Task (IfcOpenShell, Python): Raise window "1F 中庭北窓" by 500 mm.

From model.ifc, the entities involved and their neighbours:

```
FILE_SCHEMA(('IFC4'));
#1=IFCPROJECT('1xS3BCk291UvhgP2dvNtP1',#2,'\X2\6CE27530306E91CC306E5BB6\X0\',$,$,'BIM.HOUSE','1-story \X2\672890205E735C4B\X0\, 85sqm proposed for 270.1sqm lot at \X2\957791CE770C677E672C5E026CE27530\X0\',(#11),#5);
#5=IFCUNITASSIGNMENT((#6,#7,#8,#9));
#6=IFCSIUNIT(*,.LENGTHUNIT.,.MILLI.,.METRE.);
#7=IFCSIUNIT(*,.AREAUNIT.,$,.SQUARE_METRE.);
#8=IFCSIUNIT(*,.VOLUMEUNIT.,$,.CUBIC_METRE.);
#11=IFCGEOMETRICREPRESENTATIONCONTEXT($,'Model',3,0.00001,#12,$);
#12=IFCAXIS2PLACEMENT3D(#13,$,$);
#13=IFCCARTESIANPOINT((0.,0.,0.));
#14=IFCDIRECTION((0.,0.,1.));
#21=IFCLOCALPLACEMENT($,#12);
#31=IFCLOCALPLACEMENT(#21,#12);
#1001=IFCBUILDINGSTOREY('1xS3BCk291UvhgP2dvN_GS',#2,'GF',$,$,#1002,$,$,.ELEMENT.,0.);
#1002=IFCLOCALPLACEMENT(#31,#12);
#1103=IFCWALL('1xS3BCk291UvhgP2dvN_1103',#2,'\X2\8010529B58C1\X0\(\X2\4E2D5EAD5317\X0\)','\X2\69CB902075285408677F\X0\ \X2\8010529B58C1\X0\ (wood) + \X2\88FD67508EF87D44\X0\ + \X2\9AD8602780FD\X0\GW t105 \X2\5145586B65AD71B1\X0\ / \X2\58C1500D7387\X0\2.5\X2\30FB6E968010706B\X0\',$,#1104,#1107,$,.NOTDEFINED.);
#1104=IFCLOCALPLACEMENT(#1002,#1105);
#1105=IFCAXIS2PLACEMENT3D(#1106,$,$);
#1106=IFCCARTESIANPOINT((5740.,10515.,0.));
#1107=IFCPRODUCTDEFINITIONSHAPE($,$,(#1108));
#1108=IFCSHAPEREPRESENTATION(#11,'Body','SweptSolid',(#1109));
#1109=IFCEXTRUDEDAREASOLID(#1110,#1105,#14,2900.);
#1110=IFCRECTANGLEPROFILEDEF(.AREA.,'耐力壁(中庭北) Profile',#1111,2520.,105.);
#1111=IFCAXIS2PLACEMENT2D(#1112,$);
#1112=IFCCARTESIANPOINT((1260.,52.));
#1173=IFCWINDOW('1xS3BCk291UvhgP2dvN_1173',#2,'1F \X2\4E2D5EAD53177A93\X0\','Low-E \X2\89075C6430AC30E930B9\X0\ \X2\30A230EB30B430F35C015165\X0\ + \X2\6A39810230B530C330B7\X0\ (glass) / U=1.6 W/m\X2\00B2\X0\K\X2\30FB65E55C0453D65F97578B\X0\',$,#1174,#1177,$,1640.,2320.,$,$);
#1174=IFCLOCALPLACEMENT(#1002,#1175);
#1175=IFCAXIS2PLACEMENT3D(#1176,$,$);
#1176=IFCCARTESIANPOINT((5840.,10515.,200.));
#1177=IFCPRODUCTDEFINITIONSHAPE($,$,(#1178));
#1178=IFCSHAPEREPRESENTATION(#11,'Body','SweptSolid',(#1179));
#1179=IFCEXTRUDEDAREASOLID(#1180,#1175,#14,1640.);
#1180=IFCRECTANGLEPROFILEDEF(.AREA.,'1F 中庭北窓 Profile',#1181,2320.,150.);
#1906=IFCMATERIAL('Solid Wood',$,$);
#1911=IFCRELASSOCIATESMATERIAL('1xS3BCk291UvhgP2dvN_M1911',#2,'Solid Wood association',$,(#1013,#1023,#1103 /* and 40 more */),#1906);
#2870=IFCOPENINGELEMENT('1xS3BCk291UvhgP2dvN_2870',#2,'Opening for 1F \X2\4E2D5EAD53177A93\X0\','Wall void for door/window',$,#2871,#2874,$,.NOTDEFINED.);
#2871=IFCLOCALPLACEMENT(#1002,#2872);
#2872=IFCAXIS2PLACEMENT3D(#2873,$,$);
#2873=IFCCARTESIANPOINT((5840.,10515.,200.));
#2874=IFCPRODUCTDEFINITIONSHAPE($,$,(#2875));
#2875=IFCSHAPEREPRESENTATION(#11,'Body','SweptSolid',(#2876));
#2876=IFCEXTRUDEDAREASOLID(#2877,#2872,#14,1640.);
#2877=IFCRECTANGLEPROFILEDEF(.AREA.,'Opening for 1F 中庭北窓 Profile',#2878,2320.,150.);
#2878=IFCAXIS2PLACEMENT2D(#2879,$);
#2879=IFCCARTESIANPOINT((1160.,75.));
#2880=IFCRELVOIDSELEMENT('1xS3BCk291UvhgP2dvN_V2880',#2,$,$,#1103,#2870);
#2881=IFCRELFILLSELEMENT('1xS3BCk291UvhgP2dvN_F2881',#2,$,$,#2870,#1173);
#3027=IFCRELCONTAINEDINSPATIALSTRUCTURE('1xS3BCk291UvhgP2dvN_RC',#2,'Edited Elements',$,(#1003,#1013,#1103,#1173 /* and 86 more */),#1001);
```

```python
import numpy as np
import ifcopenshell
import ifcopenshell.api.geometry
import ifcopenshell.util.placement
import ifcopenshell.util.unit

model = ifcopenshell.open("model.ifc")
unit_scale = ifcopenshell.util.unit.calculate_unit_scale(model)

window = model.by_guid("1xS3BCk291UvhgP2dvN_1173")
opening = window.FillsVoids[0].RelatingOpeningElement
dz = 0.5 / unit_scale

shift = np.array([0.0, 0.0, dz])
# The window is not placed relative to its opening, so move both.
for product in (opening, window):
    matrix = ifcopenshell.util.placement.get_local_placement(product.ObjectPlacement)
    matrix[:3, 3] += shift
    ifcopenshell.api.geometry.edit_object_placement(model, product=product, matrix=matrix, is_si=False)

print(f"moved by {dz * unit_scale:+.3f} m")

model.write("model_rev.ifc")
```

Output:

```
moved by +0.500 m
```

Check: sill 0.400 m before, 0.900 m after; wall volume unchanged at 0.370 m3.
